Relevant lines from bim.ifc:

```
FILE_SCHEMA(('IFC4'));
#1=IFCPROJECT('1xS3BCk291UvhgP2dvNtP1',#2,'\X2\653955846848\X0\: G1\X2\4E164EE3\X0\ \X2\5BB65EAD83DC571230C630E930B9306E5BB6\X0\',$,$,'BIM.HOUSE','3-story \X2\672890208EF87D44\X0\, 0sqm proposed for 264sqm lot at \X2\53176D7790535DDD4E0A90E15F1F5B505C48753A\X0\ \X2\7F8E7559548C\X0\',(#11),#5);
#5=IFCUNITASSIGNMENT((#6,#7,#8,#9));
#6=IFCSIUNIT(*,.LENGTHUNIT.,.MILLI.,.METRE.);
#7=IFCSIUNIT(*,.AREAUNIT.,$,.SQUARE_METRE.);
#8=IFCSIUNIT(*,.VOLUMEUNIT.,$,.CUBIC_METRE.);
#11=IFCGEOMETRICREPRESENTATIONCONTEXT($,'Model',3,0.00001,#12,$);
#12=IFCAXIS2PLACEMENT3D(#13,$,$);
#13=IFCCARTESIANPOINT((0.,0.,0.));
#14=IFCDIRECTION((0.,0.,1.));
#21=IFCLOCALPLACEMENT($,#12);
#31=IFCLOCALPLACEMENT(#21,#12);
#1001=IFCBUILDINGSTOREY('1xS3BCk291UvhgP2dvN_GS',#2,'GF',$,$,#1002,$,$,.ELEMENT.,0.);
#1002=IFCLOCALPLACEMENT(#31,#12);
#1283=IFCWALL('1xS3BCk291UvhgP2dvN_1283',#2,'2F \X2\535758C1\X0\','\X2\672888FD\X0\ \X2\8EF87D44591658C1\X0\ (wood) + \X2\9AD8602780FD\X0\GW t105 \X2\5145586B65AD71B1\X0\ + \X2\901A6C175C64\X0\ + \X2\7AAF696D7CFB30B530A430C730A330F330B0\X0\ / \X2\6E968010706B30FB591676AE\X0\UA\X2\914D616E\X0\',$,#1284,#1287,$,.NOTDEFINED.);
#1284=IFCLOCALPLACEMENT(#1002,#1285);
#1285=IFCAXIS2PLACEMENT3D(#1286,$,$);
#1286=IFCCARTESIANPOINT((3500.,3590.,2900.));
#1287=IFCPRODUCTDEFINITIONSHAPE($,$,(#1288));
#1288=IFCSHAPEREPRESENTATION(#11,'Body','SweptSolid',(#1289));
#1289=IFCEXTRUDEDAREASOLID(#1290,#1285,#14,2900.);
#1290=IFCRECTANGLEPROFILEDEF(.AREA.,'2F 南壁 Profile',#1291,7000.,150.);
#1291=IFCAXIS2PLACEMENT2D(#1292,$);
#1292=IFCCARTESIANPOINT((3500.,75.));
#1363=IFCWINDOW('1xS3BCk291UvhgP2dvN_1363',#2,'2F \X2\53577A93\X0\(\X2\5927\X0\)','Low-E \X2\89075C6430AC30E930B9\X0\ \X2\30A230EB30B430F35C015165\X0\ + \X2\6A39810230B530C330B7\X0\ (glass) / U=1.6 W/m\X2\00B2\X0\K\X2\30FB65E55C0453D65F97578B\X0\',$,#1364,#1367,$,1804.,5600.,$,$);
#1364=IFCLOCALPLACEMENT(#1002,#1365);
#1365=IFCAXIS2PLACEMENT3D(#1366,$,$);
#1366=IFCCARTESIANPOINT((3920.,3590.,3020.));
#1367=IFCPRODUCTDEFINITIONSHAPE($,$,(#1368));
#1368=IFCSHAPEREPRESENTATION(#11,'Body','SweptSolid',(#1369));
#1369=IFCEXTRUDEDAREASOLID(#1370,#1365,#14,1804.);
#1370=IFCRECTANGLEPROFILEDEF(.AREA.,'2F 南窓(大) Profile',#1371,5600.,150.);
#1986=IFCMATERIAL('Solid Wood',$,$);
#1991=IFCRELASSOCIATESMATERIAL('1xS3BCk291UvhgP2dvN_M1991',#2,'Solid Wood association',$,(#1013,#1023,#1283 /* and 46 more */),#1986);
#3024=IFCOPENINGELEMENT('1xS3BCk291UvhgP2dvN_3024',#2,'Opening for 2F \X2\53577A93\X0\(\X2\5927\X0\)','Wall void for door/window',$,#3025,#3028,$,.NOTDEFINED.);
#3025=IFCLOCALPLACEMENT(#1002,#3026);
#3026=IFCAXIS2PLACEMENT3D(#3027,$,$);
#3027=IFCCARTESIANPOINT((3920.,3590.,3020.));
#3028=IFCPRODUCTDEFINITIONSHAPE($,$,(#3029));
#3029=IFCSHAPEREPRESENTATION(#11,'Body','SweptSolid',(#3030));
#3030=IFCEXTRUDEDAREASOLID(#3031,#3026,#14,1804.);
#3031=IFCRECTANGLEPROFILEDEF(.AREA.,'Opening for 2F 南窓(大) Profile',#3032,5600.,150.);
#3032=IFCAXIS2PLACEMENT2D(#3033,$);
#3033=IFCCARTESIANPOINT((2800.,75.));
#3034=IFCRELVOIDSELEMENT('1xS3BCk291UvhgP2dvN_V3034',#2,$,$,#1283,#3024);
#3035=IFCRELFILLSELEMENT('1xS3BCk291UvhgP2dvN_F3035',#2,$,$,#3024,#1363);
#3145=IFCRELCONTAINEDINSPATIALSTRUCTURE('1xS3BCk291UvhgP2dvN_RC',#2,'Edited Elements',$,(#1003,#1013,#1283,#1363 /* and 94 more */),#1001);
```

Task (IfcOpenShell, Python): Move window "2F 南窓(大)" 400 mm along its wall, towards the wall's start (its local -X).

```python
import ifcopenshell
import ifcopenshell.api.geometry
import ifcopenshell.util.placement
import ifcopenshell.util.unit

model = ifcopenshell.open("bim.ifc")
unit_scale = ifcopenshell.util.unit.calculate_unit_scale(model)

window = model.by_guid("1xS3BCk291UvhgP2dvN_1363")
opening = window.FillsVoids[0].RelatingOpeningElement
wall = opening.VoidsElements[0].RelatingBuildingElement

wall_matrix = ifcopenshell.util.placement.get_local_placement(wall.ObjectPlacement)
shift = wall_matrix[:3, 0] * -0.4 / unit_scale
before = ifcopenshell.util.placement.get_local_placement(window.ObjectPlacement)[:3, 3].copy()

# The window is not placed relative to its opening, so move both.
for product in (opening, window):
    matrix = ifcopenshell.util.placement.get_local_placement(product.ObjectPlacement)
    matrix[:3, 3] += shift
    ifcopenshell.api.geometry.edit_object_placement(model, product=product, matrix=matrix, is_si=False)

after = ifcopenshell.util.placement.get_local_placement(window.ObjectPlacement)[:3, 3]
print("window moved by", (after - before).round(3) + 0.0)

model.write("bim_rev.ifc")
```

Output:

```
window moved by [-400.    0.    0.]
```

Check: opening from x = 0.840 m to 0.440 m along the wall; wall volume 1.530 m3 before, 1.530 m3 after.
